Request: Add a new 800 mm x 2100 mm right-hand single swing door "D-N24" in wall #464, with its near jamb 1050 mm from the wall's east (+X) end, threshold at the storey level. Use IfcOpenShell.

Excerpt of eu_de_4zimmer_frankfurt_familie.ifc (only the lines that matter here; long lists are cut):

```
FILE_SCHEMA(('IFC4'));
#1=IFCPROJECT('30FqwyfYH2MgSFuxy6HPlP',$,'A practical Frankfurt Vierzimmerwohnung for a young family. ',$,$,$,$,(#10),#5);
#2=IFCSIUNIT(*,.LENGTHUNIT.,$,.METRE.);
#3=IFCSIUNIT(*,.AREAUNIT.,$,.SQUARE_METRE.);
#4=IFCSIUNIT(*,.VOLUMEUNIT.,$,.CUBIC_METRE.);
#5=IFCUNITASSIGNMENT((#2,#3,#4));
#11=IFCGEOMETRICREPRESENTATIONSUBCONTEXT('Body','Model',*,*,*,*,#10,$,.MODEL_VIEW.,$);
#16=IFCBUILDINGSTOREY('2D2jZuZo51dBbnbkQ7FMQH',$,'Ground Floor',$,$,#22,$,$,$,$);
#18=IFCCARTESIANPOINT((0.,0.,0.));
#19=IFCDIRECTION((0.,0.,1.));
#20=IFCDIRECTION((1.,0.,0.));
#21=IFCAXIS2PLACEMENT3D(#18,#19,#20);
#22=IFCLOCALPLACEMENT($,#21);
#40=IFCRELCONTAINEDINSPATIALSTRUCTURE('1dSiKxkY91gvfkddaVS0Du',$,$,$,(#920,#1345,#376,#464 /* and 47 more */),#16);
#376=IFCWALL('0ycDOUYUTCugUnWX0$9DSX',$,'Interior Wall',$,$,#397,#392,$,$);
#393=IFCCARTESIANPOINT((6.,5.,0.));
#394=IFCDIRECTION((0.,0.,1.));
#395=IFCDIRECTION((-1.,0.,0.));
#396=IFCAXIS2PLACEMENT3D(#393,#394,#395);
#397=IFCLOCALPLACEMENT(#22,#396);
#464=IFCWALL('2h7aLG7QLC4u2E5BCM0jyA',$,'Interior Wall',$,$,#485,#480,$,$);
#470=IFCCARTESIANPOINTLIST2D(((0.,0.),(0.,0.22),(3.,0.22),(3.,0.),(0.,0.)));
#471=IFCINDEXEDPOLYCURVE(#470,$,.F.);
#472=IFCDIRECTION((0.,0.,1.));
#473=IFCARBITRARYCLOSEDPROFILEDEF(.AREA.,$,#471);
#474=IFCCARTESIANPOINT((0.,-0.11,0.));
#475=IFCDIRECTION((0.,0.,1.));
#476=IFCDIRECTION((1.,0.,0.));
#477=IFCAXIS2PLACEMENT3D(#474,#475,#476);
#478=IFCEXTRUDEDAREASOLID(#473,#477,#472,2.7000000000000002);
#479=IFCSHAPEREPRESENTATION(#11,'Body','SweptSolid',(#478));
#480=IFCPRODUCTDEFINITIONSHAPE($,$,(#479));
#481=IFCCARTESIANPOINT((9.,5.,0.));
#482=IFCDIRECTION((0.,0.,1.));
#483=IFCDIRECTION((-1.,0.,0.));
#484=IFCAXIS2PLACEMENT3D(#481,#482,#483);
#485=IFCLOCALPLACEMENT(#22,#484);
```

```python
import numpy as np
import ifcopenshell
import ifcopenshell.api.feature
import ifcopenshell.api.geometry
import ifcopenshell.api.root
import ifcopenshell.api.spatial
import ifcopenshell.geom
import ifcopenshell.util.element
import ifcopenshell.util.placement
import ifcopenshell.util.representation
import ifcopenshell.util.shape
import ifcopenshell.util.unit

model = ifcopenshell.open("eu_de_4zimmer_frankfurt_familie.ifc")
unit_scale = ifcopenshell.util.unit.calculate_unit_scale(model)
settings = ifcopenshell.geom.settings()


def volume(element):
    """Net volume in cubic metres, openings subtracted."""
    shape = ifcopenshell.geom.create_shape(settings, element)
    return ifcopenshell.util.shape.get_volume(shape.geometry)


wall = model.by_guid("2h7aLG7QLC4u2E5BCM0jyA")
storey = ifcopenshell.util.element.get_container(wall, ifc_class="IfcBuildingStorey")
context = ifcopenshell.util.representation.get_context(model, "Model", "Body", "MODEL_VIEW")
before = volume(wall)

width, height, from_end, sill = 0.8, 2.1, 1.05, 0.0  # metres

# The wall runs along its own X axis, and the end named is its -X end.
wall_shape = ifcopenshell.geom.create_shape(settings, wall)
x, y, z = ifcopenshell.util.shape.get_vertices(wall_shape.geometry).T
start = x.min() + from_end
face, thickness = float(y.min()), float(y.max() - y.min())
wall_matrix = ifcopenshell.util.placement.get_local_placement(wall.ObjectPlacement)
level = ifcopenshell.util.placement.get_local_placement(storey.ObjectPlacement)[2, 3]


def in_wall(x, y):
    """Placement at x, y metres in the wall's axes, at sill height."""
    matrix = wall_matrix.copy()
    matrix[:, 3] = wall_matrix @ np.array([x / unit_scale, y / unit_scale, 0.0, 1.0])
    matrix[2, 3] = level + sill / unit_scale
    return matrix


# Opening: a box that overshoots both wall faces by 50 mm.
opening = ifcopenshell.api.root.create_entity(model, ifc_class="IfcOpeningElement", predefined_type="OPENING")
box = ifcopenshell.api.geometry.add_wall_representation(
    model, context=context, length=width, height=height, thickness=thickness + 0.1
)
ifcopenshell.api.geometry.assign_representation(model, product=opening, representation=box)
ifcopenshell.api.geometry.edit_object_placement(model, product=opening, matrix=in_wall(start, face - 0.05), is_si=False)
ifcopenshell.api.feature.add_feature(model, feature=opening, element=wall)

door = ifcopenshell.api.root.create_entity(model, ifc_class="IfcDoor", name="D-N24", predefined_type="DOOR")
door.OverallWidth, door.OverallHeight = width / unit_scale, height / unit_scale
door.OperationType = "SINGLE_SWING_RIGHT"
body = ifcopenshell.api.geometry.add_door_representation(
    model,
    context=context,
    overall_width=door.OverallWidth,
    overall_height=door.OverallHeight,
    operation_type="SINGLE_SWING_RIGHT",
    lining_properties={"LiningDepth": thickness / unit_scale, "ThresholdDepth": thickness / unit_scale},
)
ifcopenshell.api.geometry.assign_representation(model, product=door, representation=body)
ifcopenshell.api.spatial.assign_container(model, products=[door], relating_structure=storey)
ifcopenshell.api.feature.add_filling(model, opening=opening, element=door)

# The lining spans the wall, so the door starts at the wall face.
ifcopenshell.api.geometry.edit_object_placement(model, product=door, matrix=in_wall(start, face), is_si=False)

after = volume(wall)

print(f"wall volume {before:.3f} -> {after:.3f} m3")

model.write("eu_de_4zimmer_frankfurt_familie-out.ifc")
```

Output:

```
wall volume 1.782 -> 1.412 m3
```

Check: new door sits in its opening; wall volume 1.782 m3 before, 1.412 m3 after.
